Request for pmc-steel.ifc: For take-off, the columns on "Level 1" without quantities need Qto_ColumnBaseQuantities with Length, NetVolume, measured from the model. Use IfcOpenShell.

First a look at what the model holds.

```python
import ifcopenshell
import ifcopenshell.util.element
import ifcopenshell.util.unit

model = ifcopenshell.open("pmc-steel.ifc")
print(model.schema)
for unit_type in ("LENGTHUNIT", "AREAUNIT", "VOLUMEUNIT"):
    print(unit_type, ifcopenshell.util.unit.calculate_unit_scale(model, unit_type))
storey = next(s for s in model.by_type("IfcBuildingStorey") if s.Name == "Level 1")
columns = [e for e in ifcopenshell.util.element.get_decomposition(storey) if e.is_a("IfcColumn")]
for e in sorted(columns, key=lambda e: e.id()):
    print(e.id(), e.is_a(), e.Name, list(ifcopenshell.util.element.get_psets(e, qtos_only=True)), sep=" | ")
```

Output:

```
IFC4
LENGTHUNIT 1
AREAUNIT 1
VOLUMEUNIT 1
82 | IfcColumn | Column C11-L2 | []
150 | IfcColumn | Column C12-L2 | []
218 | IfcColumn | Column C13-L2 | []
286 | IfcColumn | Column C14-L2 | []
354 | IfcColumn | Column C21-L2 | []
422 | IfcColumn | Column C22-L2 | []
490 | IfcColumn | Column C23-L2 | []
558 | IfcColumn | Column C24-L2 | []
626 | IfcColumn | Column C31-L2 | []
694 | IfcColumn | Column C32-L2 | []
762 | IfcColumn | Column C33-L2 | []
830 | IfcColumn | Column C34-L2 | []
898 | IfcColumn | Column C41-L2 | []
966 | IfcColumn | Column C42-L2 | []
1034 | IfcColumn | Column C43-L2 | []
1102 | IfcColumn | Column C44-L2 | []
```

```python
import ifcopenshell
import ifcopenshell.api.pset
import ifcopenshell.geom
import ifcopenshell.util.element
import ifcopenshell.util.shape
import ifcopenshell.util.unit

model = ifcopenshell.open("pmc-steel.ifc")
unit_scale = ifcopenshell.util.unit.calculate_unit_scale(model)
volume_scale = ifcopenshell.util.unit.calculate_unit_scale(model, "VOLUMEUNIT")
settings = ifcopenshell.geom.settings()

storey = next(s for s in model.by_type("IfcBuildingStorey") if s.Name == "Level 1")
columns = [e for e in ifcopenshell.util.element.get_decomposition(storey) if e.is_a("IfcColumn")]

for e in sorted(columns, key=lambda e: e.id()):
    if ifcopenshell.util.element.get_psets(e, qtos_only=True, should_inherit=False):
        continue
    # Geometry comes back in metres, in the element's own axes.
    shape = ifcopenshell.geom.create_shape(settings, e)
    values = {
        "Length": ifcopenshell.util.shape.get_z(shape.geometry) / unit_scale,
        "NetVolume": ifcopenshell.util.shape.get_volume(shape.geometry) / volume_scale,
    }
    qto = ifcopenshell.api.pset.add_qto(model, product=e, name="Qto_ColumnBaseQuantities")
    ifcopenshell.api.pset.edit_qto(model, qto=qto, properties=values)
    print(e.id(), {k: round(v, 3) for k, v in values.items()})

model.write("pmc-steel_rev.ifc")
```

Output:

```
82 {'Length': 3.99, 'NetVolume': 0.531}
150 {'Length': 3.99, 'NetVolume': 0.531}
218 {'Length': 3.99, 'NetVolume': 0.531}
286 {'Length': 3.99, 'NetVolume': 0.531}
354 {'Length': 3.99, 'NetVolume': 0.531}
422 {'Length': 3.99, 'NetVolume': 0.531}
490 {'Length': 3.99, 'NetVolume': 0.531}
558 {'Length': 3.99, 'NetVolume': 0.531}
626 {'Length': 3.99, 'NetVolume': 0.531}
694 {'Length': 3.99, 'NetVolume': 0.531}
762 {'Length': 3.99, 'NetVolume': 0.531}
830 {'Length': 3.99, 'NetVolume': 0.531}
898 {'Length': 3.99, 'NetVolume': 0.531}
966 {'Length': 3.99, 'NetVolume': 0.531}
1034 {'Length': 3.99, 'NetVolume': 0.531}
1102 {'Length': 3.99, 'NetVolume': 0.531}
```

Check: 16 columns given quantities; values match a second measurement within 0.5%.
